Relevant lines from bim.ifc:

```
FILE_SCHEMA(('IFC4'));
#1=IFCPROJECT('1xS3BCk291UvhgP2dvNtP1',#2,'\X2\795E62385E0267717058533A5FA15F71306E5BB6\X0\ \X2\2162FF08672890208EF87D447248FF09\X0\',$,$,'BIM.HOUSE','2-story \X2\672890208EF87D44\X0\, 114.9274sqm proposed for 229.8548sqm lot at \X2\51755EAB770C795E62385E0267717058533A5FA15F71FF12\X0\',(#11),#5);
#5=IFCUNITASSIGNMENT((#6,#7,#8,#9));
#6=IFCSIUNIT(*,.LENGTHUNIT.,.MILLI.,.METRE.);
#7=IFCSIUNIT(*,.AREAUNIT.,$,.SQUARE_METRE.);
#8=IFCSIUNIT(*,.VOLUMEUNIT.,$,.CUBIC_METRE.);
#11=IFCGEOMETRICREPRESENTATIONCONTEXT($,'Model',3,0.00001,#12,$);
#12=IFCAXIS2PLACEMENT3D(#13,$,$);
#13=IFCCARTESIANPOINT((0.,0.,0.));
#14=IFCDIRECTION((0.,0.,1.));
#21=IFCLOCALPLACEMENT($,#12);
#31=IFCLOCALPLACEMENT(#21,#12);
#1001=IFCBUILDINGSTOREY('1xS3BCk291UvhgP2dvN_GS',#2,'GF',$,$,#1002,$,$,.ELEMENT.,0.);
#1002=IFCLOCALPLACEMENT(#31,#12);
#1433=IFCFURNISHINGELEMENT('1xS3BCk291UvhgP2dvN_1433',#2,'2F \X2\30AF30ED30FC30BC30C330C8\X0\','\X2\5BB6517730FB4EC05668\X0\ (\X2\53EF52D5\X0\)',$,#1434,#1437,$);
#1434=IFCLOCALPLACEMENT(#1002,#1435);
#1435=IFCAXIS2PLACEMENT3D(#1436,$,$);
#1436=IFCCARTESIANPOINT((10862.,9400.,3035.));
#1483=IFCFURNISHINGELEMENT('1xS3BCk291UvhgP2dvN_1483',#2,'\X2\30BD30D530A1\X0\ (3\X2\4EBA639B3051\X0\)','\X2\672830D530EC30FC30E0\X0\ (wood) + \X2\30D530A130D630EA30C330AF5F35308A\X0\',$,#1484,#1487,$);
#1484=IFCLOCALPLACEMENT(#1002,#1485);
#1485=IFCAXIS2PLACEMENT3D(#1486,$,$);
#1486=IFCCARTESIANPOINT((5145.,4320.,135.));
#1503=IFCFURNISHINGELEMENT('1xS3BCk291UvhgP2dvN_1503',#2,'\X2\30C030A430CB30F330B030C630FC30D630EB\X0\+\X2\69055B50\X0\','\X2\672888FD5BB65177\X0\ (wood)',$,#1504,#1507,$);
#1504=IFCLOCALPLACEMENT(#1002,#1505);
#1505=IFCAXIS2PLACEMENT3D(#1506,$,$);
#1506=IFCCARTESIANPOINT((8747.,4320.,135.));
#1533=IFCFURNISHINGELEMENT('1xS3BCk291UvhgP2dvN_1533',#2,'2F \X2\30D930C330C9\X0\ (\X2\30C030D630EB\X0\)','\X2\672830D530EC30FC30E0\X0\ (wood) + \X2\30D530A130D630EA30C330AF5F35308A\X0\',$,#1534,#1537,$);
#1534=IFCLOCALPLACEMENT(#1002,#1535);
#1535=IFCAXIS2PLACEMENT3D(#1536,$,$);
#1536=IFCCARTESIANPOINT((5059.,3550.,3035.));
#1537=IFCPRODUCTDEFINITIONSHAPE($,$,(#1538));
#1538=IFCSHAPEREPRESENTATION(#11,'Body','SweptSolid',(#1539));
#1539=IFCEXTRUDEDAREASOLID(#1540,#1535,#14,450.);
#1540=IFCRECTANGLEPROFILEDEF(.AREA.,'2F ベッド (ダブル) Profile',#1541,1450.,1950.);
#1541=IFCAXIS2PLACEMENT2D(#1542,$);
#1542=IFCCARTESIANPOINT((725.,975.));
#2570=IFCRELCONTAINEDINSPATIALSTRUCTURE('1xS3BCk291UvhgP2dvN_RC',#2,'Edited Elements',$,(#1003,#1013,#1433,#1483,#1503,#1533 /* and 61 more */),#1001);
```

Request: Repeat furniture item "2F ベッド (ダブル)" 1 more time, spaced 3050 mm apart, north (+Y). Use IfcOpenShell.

```python
import numpy as np
import ifcopenshell
import ifcopenshell.api.geometry
import ifcopenshell.api.root
import ifcopenshell.util.element
import ifcopenshell.util.placement
import ifcopenshell.util.unit

model = ifcopenshell.open("bim.ifc")
unit_scale = ifcopenshell.util.unit.calculate_unit_scale(model)


def reuse_history(source, copy):
    """copy_class also copies each property set's owner history, people and application; keep the originals."""
    for rel in copy.IsDefinedBy:
        if rel.is_a("IfcRelDefinesByProperties") and (history := rel.RelatingPropertyDefinition.OwnerHistory):
            rel.RelatingPropertyDefinition.OwnerHistory = source.OwnerHistory
            ifcopenshell.util.element.remove_deep2(model, history)


source = model.by_guid("1xS3BCk291UvhgP2dvN_1533")
base = ifcopenshell.util.placement.get_local_placement(source.ObjectPlacement)
step = np.array([0.0, 1.0, 0.0]) * 3.05 / unit_scale

for i in range(1, 2):
    copy = ifcopenshell.api.root.copy_class(model, product=source)
    copy.Representation = ifcopenshell.util.element.copy_deep(
        model, source.Representation, exclude=["IfcGeometricRepresentationContext", "IfcRepresentationMap"]
    )
    reuse_history(source, copy)
    matrix = base.copy()
    matrix[:3, 3] += i * step
    print("added at", matrix[:3, 3].round(3) + 0.0)
    ifcopenshell.api.geometry.edit_object_placement(model, product=copy, matrix=matrix, is_si=False)

model.write("bim-out.ifc")
```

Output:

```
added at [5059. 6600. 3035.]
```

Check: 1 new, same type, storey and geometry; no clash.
